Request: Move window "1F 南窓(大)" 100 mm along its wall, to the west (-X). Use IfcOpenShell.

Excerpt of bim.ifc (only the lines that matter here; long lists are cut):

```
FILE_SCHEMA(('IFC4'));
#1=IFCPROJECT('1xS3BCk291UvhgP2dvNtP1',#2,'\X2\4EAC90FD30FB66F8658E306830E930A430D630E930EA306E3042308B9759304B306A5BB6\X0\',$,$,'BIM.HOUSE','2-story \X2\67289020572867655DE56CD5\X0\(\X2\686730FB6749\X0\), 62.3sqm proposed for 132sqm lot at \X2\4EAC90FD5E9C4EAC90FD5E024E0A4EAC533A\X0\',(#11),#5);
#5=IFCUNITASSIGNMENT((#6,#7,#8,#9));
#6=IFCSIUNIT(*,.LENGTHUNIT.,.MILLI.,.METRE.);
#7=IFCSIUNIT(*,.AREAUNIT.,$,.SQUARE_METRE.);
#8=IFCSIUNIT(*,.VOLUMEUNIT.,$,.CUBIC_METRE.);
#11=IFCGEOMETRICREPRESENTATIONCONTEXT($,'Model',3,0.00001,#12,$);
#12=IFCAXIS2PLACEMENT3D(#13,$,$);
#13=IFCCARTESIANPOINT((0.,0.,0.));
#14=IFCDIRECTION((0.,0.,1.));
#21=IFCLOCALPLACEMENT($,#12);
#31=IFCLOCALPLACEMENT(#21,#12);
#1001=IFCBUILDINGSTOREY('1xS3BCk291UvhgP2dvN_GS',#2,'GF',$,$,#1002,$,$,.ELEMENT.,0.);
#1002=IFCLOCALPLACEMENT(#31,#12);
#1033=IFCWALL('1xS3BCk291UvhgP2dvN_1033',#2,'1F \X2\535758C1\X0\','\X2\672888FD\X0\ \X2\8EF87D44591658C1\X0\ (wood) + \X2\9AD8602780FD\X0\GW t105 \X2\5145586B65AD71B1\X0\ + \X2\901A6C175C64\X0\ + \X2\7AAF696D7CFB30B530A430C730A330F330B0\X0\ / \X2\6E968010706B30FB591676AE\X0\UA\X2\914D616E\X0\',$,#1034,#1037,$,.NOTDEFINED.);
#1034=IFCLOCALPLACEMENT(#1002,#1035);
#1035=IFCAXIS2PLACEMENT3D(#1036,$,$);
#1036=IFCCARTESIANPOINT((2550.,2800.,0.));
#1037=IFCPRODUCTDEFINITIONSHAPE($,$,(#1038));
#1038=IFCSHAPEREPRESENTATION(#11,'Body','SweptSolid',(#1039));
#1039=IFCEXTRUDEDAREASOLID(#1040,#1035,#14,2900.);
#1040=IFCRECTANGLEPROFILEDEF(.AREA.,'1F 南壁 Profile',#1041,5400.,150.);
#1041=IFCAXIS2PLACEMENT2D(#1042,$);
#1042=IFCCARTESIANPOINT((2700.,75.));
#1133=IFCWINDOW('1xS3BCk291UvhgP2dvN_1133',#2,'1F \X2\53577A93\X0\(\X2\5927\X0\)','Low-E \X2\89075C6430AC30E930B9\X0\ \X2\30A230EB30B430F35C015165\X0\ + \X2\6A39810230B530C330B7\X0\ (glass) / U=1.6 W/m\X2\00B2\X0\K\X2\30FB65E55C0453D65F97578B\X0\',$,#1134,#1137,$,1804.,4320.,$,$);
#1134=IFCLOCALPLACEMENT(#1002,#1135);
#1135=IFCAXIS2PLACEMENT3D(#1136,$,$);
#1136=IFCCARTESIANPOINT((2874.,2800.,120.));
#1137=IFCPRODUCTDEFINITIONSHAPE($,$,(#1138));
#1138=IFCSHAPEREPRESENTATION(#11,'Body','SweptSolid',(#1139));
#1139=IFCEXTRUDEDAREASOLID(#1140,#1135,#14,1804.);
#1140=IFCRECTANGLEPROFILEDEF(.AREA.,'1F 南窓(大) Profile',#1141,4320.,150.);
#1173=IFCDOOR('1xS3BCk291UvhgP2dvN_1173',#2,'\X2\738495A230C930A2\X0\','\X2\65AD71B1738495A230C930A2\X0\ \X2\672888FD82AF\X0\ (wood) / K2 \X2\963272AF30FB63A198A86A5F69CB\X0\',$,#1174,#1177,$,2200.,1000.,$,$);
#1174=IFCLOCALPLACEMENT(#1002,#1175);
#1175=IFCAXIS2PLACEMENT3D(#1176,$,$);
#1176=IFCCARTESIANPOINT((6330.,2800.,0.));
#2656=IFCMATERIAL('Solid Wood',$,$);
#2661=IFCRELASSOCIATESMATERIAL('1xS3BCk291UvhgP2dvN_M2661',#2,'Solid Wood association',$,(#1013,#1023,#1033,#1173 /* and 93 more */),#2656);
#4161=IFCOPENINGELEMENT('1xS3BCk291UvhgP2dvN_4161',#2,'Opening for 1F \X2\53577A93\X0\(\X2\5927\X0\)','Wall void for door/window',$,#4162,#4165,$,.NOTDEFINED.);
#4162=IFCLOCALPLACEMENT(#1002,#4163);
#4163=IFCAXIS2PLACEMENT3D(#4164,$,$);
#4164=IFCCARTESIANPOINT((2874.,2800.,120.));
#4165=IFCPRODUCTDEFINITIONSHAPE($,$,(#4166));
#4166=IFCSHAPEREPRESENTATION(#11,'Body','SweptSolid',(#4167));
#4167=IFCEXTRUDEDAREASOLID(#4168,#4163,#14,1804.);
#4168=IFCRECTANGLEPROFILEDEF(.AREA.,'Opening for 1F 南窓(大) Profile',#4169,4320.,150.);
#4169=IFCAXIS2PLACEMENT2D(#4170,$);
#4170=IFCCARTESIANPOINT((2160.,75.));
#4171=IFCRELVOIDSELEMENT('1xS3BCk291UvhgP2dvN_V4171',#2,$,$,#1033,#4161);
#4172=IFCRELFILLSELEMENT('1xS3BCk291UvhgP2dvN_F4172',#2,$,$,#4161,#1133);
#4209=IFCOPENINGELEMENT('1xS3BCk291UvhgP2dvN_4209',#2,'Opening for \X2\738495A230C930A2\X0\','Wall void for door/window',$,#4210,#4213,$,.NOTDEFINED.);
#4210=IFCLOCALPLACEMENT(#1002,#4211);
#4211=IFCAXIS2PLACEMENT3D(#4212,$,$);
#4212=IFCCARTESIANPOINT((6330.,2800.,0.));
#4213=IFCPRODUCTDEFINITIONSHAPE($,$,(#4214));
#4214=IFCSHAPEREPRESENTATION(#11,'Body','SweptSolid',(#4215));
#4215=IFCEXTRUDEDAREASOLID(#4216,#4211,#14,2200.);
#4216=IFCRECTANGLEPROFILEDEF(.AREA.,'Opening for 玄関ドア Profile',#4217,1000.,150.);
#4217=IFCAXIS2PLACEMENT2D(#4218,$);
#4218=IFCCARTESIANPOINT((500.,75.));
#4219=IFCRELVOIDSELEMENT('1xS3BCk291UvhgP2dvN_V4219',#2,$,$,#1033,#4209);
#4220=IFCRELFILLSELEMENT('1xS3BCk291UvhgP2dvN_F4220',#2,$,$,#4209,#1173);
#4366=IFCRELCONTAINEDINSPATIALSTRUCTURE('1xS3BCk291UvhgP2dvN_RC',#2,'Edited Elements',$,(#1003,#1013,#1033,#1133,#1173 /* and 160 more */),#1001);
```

```python
import ifcopenshell
import ifcopenshell.api.geometry
import ifcopenshell.util.placement
import ifcopenshell.util.unit

model = ifcopenshell.open("bim.ifc")
unit_scale = ifcopenshell.util.unit.calculate_unit_scale(model)

window = model.by_guid("1xS3BCk291UvhgP2dvN_1133")
opening = window.FillsVoids[0].RelatingOpeningElement
wall = opening.VoidsElements[0].RelatingBuildingElement

wall_matrix = ifcopenshell.util.placement.get_local_placement(wall.ObjectPlacement)
shift = wall_matrix[:3, 0] * -0.1 / unit_scale
before = ifcopenshell.util.placement.get_local_placement(window.ObjectPlacement)[:3, 3].copy()

# The window is not placed relative to its opening, so move both.
for product in (opening, window):
    matrix = ifcopenshell.util.placement.get_local_placement(product.ObjectPlacement)
    matrix[:3, 3] += shift
    ifcopenshell.api.geometry.edit_object_placement(model, product=product, matrix=matrix, is_si=False)

after = ifcopenshell.util.placement.get_local_placement(window.ObjectPlacement)[:3, 3]
print("window moved by", (after - before).round(3) + 0.0)

model.write("bim_updated.ifc")
```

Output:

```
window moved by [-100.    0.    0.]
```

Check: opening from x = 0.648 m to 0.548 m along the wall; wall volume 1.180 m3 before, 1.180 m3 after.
